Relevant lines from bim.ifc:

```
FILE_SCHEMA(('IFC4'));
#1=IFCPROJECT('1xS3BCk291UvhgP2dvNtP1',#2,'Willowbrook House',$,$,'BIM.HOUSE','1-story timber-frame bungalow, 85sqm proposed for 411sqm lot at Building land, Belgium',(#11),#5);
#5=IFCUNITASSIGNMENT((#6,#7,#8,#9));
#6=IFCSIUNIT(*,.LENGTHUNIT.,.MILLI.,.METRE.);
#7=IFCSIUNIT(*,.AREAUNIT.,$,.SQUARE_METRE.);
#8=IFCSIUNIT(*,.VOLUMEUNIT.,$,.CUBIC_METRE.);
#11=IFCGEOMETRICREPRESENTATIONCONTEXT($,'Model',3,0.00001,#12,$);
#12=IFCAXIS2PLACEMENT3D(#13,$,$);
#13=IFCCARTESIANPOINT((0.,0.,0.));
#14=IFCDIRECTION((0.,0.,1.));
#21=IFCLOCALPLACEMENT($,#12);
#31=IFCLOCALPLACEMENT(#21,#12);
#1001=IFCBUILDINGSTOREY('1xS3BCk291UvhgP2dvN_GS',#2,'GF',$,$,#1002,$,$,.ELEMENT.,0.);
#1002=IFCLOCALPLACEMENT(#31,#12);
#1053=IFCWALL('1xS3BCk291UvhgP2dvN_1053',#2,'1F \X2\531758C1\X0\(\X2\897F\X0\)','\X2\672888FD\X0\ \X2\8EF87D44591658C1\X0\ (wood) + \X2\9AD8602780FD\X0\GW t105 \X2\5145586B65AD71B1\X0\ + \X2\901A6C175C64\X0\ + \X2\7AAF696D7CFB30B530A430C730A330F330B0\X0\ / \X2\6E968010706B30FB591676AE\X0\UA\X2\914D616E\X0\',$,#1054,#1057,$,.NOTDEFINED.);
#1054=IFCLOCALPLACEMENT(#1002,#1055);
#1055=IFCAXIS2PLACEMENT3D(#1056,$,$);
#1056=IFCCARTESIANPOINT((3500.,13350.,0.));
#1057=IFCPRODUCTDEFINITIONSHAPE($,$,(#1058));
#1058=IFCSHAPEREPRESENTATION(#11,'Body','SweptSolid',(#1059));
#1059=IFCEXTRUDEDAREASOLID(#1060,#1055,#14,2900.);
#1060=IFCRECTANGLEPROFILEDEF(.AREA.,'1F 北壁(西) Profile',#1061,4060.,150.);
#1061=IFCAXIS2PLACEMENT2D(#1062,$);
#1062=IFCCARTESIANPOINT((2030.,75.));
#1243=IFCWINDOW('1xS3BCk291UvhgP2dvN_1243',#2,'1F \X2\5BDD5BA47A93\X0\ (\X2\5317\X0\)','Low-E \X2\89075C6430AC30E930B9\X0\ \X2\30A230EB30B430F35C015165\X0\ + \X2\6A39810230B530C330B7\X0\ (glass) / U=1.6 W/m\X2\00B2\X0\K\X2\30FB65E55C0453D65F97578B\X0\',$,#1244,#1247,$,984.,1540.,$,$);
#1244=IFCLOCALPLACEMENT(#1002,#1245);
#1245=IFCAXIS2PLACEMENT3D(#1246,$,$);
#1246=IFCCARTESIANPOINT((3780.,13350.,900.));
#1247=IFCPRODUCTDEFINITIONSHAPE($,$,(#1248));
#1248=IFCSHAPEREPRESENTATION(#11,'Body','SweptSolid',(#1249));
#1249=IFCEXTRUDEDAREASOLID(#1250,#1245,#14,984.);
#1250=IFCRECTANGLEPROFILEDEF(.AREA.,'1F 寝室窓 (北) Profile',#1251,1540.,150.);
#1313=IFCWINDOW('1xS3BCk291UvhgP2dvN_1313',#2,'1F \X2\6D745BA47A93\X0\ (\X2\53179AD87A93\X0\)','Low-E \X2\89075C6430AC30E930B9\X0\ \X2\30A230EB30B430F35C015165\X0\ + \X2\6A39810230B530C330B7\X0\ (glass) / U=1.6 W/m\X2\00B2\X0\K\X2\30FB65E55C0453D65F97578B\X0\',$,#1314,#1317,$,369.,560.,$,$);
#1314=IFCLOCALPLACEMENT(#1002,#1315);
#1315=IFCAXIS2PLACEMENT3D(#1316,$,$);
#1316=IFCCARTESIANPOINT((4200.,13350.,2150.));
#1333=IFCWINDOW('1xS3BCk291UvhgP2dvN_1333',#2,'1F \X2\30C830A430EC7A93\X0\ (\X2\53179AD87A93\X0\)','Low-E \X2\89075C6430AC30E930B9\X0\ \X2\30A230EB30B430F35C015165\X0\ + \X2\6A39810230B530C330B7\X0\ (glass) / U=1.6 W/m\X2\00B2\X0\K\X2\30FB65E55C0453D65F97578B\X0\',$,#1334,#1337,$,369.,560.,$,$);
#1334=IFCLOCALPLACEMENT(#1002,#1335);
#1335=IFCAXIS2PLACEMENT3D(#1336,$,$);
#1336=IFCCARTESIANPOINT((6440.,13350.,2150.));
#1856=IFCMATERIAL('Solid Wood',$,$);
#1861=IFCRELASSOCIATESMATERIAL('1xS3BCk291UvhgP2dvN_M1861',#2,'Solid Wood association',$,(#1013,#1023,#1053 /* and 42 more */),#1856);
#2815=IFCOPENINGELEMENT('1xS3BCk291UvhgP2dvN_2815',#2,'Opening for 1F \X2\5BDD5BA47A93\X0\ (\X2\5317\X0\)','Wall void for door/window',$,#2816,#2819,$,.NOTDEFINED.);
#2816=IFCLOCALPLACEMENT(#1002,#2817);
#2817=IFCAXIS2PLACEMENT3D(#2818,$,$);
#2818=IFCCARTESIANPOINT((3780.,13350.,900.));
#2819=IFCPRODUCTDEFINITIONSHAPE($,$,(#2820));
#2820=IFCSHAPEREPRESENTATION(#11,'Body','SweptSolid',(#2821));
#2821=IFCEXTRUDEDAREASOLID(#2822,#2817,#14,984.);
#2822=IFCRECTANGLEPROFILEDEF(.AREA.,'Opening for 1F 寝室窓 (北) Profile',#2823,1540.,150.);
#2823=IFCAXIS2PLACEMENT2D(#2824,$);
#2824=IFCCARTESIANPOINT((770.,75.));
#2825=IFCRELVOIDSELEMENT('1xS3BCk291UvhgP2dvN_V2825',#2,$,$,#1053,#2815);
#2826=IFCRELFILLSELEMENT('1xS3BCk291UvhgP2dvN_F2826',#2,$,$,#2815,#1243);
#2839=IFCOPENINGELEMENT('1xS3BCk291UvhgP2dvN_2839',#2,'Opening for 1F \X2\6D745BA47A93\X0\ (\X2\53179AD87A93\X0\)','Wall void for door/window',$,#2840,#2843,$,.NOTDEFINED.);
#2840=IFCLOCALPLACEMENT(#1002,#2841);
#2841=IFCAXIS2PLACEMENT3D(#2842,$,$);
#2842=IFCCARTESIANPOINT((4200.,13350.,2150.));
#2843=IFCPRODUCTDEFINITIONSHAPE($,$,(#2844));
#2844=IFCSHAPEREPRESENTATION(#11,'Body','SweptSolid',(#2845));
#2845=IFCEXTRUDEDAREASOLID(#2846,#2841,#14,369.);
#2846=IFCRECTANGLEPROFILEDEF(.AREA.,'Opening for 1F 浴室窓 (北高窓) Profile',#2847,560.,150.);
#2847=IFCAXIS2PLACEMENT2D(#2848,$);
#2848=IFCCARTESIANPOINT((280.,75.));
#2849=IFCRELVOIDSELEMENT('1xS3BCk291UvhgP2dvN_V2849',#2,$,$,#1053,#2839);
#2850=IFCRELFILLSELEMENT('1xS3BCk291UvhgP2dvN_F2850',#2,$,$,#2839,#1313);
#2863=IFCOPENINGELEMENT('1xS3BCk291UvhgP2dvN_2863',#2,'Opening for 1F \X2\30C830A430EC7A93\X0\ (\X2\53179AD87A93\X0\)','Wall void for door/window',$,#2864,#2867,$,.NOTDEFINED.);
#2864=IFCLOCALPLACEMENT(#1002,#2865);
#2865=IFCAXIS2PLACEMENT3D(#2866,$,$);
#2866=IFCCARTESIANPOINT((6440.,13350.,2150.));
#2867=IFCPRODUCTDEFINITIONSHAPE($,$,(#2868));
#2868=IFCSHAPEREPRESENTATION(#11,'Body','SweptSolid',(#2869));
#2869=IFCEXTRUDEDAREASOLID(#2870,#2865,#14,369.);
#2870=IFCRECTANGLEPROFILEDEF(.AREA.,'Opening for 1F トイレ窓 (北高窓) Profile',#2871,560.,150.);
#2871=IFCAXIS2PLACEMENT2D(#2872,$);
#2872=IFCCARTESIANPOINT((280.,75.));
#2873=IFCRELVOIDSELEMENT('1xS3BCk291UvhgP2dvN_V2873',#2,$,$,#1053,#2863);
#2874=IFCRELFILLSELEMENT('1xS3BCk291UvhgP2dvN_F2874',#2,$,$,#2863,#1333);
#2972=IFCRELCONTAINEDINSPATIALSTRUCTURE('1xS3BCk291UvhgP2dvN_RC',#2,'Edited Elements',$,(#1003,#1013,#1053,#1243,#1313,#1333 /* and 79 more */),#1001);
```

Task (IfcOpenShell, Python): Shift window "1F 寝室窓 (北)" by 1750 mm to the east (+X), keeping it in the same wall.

```python
import ifcopenshell
import ifcopenshell.api.geometry
import ifcopenshell.util.placement

model = ifcopenshell.open("bim.ifc")

window = model.by_guid("1xS3BCk291UvhgP2dvN_1243")
opening = window.FillsVoids[0].RelatingOpeningElement
wall = opening.VoidsElements[0].RelatingBuildingElement

wall_matrix = ifcopenshell.util.placement.get_local_placement(wall.ObjectPlacement)
shift = wall_matrix[:3, 0] * 1750.0
before = ifcopenshell.util.placement.get_local_placement(window.ObjectPlacement)[:3, 3].copy()

# The window is not placed relative to its opening, so move both.
for product in (opening, window):
    matrix = ifcopenshell.util.placement.get_local_placement(product.ObjectPlacement)
    matrix[:3, 3] += shift
    ifcopenshell.api.geometry.edit_object_placement(model, product=product, matrix=matrix, is_si=False)

after = ifcopenshell.util.placement.get_local_placement(window.ObjectPlacement)[:3, 3]
print("window moved by", (after - before).round(3) + 0.0)

model.write("bim_updated.ifc")
```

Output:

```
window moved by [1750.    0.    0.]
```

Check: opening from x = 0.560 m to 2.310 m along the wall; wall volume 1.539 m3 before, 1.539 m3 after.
